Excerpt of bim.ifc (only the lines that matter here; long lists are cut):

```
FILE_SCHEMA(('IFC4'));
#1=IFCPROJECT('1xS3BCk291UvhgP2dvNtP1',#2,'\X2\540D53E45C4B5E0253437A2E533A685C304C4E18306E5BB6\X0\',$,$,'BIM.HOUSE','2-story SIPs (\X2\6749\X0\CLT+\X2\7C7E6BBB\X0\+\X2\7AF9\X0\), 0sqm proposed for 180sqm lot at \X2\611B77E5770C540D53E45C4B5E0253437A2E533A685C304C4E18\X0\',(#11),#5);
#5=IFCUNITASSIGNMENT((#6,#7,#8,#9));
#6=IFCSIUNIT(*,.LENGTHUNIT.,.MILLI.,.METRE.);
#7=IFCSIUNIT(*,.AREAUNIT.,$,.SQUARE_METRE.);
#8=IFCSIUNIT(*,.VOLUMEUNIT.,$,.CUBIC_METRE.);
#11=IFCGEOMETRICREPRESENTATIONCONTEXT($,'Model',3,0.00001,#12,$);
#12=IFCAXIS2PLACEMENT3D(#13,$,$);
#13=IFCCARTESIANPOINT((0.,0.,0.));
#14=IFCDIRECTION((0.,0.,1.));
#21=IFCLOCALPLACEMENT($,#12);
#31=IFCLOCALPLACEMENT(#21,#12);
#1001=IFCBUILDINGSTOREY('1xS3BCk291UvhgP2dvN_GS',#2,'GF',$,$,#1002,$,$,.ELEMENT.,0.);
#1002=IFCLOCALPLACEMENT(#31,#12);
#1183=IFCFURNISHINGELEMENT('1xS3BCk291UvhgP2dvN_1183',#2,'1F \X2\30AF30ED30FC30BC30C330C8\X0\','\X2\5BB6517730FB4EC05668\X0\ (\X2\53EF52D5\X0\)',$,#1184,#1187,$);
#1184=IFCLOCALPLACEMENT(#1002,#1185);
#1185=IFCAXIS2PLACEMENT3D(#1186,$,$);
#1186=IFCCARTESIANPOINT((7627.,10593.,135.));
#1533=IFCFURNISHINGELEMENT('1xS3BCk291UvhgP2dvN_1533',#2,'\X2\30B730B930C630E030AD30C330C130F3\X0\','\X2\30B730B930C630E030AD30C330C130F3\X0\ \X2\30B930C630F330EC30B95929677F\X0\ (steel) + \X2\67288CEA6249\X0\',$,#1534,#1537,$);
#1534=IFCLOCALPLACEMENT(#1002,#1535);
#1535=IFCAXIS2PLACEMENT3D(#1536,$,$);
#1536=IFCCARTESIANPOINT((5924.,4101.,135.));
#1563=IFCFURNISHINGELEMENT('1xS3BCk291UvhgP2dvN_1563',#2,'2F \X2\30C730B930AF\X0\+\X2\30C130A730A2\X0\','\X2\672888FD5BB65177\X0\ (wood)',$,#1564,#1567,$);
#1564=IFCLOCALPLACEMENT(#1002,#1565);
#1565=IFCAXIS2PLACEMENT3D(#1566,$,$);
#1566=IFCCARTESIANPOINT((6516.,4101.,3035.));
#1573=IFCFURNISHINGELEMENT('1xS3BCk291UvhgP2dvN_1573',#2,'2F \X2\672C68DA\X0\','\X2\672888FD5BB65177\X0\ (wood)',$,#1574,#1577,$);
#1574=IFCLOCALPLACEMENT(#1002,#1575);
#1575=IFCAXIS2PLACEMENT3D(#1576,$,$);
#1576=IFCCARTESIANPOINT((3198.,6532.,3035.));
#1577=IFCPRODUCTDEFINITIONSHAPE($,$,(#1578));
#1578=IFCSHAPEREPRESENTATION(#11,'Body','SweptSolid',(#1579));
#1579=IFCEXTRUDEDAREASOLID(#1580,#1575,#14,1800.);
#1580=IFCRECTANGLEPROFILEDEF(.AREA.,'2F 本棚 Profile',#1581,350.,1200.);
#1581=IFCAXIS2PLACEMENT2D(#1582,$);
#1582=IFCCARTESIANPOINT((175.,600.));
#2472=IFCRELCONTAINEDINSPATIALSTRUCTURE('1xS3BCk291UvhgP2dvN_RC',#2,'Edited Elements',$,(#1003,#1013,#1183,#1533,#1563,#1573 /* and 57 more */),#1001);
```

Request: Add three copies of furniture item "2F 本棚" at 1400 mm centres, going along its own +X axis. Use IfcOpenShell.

```python
import ifcopenshell
import ifcopenshell.api.geometry
import ifcopenshell.api.root
import ifcopenshell.util.element
import ifcopenshell.util.placement
import ifcopenshell.util.unit

model = ifcopenshell.open("bim.ifc")
unit_scale = ifcopenshell.util.unit.calculate_unit_scale(model)


def reuse_history(source, copy):
    """copy_class also copies each property set's owner history, people and application; keep the originals."""
    for rel in copy.IsDefinedBy:
        if rel.is_a("IfcRelDefinesByProperties") and (history := rel.RelatingPropertyDefinition.OwnerHistory):
            rel.RelatingPropertyDefinition.OwnerHistory = source.OwnerHistory
            ifcopenshell.util.element.remove_deep2(model, history)


source = model.by_guid("1xS3BCk291UvhgP2dvN_1573")
base = ifcopenshell.util.placement.get_local_placement(source.ObjectPlacement)
step = base[:3, 0] * 1.4 / unit_scale

for i in range(1, 4):
    copy = ifcopenshell.api.root.copy_class(model, product=source)
    copy.Representation = ifcopenshell.util.element.copy_deep(
        model, source.Representation, exclude=["IfcGeometricRepresentationContext", "IfcRepresentationMap"]
    )
    reuse_history(source, copy)
    matrix = base.copy()
    matrix[:3, 3] += i * step
    print("added at", matrix[:3, 3].round(3) + 0.0)
    ifcopenshell.api.geometry.edit_object_placement(model, product=copy, matrix=matrix, is_si=False)

model.write("bim_updated.ifc")
```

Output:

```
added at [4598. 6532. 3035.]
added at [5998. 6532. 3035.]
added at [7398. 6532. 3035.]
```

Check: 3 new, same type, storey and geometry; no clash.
